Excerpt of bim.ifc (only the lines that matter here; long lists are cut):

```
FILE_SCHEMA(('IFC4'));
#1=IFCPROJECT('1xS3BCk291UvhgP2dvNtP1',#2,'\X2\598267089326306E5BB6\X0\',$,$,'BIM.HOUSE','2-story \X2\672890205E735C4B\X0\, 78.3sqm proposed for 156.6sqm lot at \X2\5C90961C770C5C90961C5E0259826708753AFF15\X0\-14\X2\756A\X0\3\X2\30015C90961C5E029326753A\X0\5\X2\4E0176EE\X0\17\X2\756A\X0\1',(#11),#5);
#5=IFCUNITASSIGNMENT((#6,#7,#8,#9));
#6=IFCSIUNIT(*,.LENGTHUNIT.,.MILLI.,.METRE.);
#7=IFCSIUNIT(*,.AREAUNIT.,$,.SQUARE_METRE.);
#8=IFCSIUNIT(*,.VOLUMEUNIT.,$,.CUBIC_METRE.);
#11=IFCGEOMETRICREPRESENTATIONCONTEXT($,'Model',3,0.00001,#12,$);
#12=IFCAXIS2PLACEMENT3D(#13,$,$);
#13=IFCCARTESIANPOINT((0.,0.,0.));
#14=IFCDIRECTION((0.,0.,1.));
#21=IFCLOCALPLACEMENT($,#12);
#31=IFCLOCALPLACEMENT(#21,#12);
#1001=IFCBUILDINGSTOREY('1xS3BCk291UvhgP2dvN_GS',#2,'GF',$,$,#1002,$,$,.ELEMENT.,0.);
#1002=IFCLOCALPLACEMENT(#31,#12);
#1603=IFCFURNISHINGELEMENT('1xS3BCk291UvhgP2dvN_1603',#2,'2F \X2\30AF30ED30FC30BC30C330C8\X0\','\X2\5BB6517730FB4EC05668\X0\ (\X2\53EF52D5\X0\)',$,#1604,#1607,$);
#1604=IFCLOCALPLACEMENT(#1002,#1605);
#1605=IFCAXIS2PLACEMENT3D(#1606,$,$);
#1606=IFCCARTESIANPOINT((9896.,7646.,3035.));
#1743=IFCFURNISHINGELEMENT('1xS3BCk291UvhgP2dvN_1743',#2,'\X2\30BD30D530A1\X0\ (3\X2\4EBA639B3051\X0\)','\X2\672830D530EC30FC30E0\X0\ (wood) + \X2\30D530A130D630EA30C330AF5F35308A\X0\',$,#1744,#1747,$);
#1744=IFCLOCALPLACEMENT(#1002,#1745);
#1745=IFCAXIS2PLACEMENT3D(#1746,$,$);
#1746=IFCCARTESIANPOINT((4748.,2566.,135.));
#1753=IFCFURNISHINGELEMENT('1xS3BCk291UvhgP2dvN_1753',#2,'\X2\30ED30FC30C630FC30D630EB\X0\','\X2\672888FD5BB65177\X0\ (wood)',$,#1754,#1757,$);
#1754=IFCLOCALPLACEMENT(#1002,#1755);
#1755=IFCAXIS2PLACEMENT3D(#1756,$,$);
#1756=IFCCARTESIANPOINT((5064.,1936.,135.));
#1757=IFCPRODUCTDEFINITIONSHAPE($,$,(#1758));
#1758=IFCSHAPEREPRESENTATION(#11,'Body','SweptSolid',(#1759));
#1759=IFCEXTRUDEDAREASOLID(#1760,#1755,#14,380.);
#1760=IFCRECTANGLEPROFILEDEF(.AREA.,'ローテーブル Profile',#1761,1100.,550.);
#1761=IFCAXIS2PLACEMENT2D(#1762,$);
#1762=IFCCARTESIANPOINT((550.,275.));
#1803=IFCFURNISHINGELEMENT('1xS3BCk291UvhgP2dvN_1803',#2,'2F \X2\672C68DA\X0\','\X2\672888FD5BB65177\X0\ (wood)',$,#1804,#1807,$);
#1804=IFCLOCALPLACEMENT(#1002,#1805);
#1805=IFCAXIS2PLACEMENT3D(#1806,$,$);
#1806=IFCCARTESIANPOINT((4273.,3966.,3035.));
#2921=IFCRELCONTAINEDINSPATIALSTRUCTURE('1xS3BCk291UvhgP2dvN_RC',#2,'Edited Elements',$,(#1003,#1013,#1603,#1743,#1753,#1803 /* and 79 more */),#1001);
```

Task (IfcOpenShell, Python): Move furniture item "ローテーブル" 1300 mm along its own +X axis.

```python
import ifcopenshell
import ifcopenshell.api.geometry
import ifcopenshell.util.placement
import ifcopenshell.util.unit

model = ifcopenshell.open("bim.ifc")
unit_scale = ifcopenshell.util.unit.calculate_unit_scale(model)

item = model.by_guid("1xS3BCk291UvhgP2dvN_1753")
matrix = ifcopenshell.util.placement.get_local_placement(item.ObjectPlacement)
matrix[:3, 3] += matrix[:3, 0] * 1.3 / unit_scale
ifcopenshell.api.geometry.edit_object_placement(model, product=item, matrix=matrix, is_si=False)

print(ifcopenshell.util.placement.get_local_placement(item.ObjectPlacement).round(3) + 0.0)

model.write("bim-out.ifc")
```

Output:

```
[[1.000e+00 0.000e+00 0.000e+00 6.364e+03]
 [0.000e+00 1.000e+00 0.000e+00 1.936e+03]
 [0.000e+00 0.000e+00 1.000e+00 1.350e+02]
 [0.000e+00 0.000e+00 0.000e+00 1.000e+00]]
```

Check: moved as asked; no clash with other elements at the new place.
